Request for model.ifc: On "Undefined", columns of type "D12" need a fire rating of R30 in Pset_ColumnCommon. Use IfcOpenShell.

First a look at what the model holds.

```python
import ifcopenshell
import ifcopenshell.util.element

model = ifcopenshell.open("model.ifc")
print(model.schema)
storey = next(s for s in model.by_type("IfcBuildingStorey") if s.Name == "Undefined")
columns = [e for e in ifcopenshell.util.element.get_decomposition(storey) if e.is_a("IfcColumn")]
seen = {}
for e in columns:
    element_type = ifcopenshell.util.element.get_type(e)
    key = (element_type.Name if element_type != e and element_type else None, ifcopenshell.util.element.get_pset(e, "Pset_ColumnCommon", "FireRating"))
    seen[key] = seen.get(key, 0) + 1
for (name, value), count in sorted(seen.items(), key=str):
    print(count, "x", name, "|", value)
```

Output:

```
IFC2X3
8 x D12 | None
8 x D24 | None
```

```python
import ifcopenshell
import ifcopenshell.api.pset
import ifcopenshell.util.element

model = ifcopenshell.open("model.ifc")

storey = next(s for s in model.by_type("IfcBuildingStorey") if s.Name == "Undefined")
columns = [e for e in ifcopenshell.util.element.get_decomposition(storey) if e.is_a("IfcColumn")]

count = 0
for e in columns:
    element_type = ifcopenshell.util.element.get_type(e)
    if element_type in (None, e) or element_type.Name != "D12":
        continue
    # add_pset returns the element's existing set when there is one.
    pset = ifcopenshell.api.pset.add_pset(model, product=e, name="Pset_ColumnCommon")
    ifcopenshell.api.pset.edit_pset(model, pset=pset, properties={"FireRating": "R30"})
    count += 1

print(count, "columns updated")

model.write("model_updated.ifc")
```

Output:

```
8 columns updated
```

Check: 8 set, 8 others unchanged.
